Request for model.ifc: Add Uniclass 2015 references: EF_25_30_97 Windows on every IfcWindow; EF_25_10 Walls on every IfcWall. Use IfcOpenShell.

First a look at what the model holds.

```python
import ifcopenshell

model = ifcopenshell.open("model.ifc")
print(model.schema)
print("classifications:", [c.Name for c in model.by_type("IfcClassification")])
for ifc_class in ("IfcDoor", "IfcRoof", "IfcStair", "IfcWall", "IfcWindow"):
    print(ifc_class, len(model.by_type(ifc_class)))
```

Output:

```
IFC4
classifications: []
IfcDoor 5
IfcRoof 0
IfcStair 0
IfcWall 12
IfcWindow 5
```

```python
import ifcopenshell
import ifcopenshell.api.classification

model = ifcopenshell.open("model.ifc")

system = ifcopenshell.api.classification.add_classification(model, classification="Uniclass 2015")

codes = {
    "IfcWindow": ("EF_25_30_97", "Windows"),
    "IfcWall": ("EF_25_10", "Walls"),
}
for ifc_class, (code, name) in codes.items():
    products = model.by_type(ifc_class)
    ifcopenshell.api.classification.add_reference(
        model, products=products, classification=system, identification=code, name=name
    )
    print(code, len(products))

model.write("model_rev.ifc")
```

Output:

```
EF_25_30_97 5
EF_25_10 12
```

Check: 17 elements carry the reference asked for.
